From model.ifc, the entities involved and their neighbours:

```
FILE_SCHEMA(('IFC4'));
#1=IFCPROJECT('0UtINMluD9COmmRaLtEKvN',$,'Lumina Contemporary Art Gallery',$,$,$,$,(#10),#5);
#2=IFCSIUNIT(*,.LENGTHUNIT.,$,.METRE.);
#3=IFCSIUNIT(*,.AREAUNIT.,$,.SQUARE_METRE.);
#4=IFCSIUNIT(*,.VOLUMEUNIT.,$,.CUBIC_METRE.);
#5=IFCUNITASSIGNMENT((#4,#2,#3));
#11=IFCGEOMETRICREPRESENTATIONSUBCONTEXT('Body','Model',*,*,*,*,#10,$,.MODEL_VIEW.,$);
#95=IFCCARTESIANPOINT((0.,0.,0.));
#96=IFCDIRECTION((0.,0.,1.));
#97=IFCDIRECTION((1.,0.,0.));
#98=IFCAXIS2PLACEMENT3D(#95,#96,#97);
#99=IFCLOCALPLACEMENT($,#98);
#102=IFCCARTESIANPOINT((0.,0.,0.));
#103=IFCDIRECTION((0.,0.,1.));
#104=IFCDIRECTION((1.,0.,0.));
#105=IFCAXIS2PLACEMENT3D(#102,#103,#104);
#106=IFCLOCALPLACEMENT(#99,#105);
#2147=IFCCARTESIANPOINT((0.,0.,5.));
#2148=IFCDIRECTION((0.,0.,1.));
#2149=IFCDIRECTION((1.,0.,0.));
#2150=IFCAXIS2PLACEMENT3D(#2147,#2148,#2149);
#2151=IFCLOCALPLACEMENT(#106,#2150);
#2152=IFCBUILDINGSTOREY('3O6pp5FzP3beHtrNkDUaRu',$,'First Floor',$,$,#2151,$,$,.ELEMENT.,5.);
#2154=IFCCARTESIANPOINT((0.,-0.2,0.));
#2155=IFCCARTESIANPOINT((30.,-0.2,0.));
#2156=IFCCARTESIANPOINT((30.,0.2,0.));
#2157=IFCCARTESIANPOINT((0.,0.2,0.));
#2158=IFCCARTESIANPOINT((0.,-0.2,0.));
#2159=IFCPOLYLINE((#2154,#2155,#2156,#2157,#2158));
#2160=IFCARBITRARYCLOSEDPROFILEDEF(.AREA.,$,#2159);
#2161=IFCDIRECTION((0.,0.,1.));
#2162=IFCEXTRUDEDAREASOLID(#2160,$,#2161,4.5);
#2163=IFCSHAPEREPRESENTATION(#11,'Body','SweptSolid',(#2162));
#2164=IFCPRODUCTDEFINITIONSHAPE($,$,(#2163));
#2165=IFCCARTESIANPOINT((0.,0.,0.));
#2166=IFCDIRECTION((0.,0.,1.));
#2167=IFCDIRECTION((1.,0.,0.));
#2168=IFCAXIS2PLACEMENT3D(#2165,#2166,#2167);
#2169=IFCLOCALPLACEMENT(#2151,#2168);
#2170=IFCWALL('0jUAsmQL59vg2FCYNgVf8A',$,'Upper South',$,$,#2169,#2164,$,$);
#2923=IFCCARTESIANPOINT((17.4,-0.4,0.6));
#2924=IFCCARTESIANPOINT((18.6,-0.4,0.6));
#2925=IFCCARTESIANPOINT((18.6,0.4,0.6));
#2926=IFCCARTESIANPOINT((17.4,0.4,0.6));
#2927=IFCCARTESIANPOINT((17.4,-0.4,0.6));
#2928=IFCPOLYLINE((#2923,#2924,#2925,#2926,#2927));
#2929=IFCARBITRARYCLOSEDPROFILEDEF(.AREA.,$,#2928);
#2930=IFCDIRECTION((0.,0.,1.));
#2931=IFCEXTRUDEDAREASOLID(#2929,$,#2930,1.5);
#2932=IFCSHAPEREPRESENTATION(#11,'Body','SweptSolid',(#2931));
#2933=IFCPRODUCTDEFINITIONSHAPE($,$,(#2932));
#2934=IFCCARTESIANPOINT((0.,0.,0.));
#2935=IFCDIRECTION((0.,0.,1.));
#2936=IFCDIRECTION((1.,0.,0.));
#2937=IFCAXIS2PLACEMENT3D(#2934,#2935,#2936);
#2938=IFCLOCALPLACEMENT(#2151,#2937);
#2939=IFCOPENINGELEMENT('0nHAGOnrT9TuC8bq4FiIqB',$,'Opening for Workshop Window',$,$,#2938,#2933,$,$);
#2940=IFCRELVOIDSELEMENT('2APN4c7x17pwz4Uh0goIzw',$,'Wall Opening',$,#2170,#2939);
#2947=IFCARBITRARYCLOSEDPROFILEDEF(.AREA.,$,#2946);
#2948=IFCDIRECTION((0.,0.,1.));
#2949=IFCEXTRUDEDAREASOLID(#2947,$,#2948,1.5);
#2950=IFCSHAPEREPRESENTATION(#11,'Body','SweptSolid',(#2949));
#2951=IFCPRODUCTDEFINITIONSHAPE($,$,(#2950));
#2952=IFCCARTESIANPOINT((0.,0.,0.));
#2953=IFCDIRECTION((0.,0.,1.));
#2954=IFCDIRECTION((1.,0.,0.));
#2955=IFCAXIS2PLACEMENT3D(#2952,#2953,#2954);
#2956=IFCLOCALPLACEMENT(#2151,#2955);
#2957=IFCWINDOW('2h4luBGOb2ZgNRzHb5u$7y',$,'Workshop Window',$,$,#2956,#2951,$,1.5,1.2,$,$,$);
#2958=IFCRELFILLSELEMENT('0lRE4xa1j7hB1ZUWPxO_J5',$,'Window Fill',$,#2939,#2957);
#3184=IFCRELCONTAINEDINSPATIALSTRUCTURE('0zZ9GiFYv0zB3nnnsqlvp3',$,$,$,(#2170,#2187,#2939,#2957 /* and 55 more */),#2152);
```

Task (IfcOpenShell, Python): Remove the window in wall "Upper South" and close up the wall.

```python
import ifcopenshell
import ifcopenshell.api.feature
import ifcopenshell.api.root
import ifcopenshell.geom
import ifcopenshell.util.shape

model = ifcopenshell.open("model.ifc")
settings = ifcopenshell.geom.settings()


def volume(element):
    """Net volume in cubic metres, openings subtracted."""
    shape = ifcopenshell.geom.create_shape(settings, element)
    return ifcopenshell.util.shape.get_volume(shape.geometry)


window = model.by_guid("2h4luBGOb2ZgNRzHb5u$7y")
opening = window.FillsVoids[0].RelatingOpeningElement
wall = opening.VoidsElements[0].RelatingBuildingElement
before = volume(wall)

ifcopenshell.api.root.remove_product(model, product=window)
ifcopenshell.api.feature.remove_feature(model, feature=opening)

after = volume(wall)

print(f"wall volume {before:.3f} -> {after:.3f} m3")

model.write("model_v2.ifc")
```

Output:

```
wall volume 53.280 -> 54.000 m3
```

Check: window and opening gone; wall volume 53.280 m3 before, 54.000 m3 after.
